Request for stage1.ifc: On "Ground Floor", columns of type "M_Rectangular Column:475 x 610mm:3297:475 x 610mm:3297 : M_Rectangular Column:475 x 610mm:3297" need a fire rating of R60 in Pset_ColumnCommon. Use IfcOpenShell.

First a look at what the model holds.

```python
import ifcopenshell
import ifcopenshell.util.element

model = ifcopenshell.open("stage1.ifc")
print(model.schema)
storey = next(s for s in model.by_type("IfcBuildingStorey") if s.Name == "Ground Floor")
columns = [e for e in ifcopenshell.util.element.get_decomposition(storey) if e.is_a("IfcColumn")]
seen = {}
for e in columns:
    element_type = ifcopenshell.util.element.get_type(e)
    key = (element_type.Name if element_type != e and element_type else None, ifcopenshell.util.element.get_pset(e, "Pset_ColumnCommon", "FireRating"))
    seen[key] = seen.get(key, 0) + 1
for (name, value), count in sorted(seen.items(), key=str):
    print(count, "x", name, "|", value)
```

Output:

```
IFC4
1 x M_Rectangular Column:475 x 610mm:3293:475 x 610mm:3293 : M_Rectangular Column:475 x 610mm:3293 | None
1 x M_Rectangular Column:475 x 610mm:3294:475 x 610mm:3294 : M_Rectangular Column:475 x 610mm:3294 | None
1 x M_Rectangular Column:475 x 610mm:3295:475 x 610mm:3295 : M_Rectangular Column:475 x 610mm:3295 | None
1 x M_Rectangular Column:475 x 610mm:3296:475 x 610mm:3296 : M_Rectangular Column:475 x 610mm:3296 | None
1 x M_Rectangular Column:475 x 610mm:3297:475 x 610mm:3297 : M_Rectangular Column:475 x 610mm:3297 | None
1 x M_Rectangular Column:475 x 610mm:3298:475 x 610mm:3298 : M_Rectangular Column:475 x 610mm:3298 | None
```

```python
import ifcopenshell
import ifcopenshell.api.pset
import ifcopenshell.util.element

model = ifcopenshell.open("stage1.ifc")

storey = next(s for s in model.by_type("IfcBuildingStorey") if s.Name == "Ground Floor")
columns = [e for e in ifcopenshell.util.element.get_decomposition(storey) if e.is_a("IfcColumn")]

count = 0
for e in columns:
    element_type = ifcopenshell.util.element.get_type(e)
    if element_type in (None, e) or element_type.Name != "M_Rectangular Column:475 x 610mm:3297:475 x 610mm:3297 : M_Rectangular Column:475 x 610mm:3297":
        continue
    # add_pset returns the element's existing set when there is one.
    pset = ifcopenshell.api.pset.add_pset(model, product=e, name="Pset_ColumnCommon")
    ifcopenshell.api.pset.edit_pset(model, pset=pset, properties={"FireRating": "R60"})
    count += 1

print(count, "columns updated")

model.write("stage1-out.ifc")
```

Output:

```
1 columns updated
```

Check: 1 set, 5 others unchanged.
